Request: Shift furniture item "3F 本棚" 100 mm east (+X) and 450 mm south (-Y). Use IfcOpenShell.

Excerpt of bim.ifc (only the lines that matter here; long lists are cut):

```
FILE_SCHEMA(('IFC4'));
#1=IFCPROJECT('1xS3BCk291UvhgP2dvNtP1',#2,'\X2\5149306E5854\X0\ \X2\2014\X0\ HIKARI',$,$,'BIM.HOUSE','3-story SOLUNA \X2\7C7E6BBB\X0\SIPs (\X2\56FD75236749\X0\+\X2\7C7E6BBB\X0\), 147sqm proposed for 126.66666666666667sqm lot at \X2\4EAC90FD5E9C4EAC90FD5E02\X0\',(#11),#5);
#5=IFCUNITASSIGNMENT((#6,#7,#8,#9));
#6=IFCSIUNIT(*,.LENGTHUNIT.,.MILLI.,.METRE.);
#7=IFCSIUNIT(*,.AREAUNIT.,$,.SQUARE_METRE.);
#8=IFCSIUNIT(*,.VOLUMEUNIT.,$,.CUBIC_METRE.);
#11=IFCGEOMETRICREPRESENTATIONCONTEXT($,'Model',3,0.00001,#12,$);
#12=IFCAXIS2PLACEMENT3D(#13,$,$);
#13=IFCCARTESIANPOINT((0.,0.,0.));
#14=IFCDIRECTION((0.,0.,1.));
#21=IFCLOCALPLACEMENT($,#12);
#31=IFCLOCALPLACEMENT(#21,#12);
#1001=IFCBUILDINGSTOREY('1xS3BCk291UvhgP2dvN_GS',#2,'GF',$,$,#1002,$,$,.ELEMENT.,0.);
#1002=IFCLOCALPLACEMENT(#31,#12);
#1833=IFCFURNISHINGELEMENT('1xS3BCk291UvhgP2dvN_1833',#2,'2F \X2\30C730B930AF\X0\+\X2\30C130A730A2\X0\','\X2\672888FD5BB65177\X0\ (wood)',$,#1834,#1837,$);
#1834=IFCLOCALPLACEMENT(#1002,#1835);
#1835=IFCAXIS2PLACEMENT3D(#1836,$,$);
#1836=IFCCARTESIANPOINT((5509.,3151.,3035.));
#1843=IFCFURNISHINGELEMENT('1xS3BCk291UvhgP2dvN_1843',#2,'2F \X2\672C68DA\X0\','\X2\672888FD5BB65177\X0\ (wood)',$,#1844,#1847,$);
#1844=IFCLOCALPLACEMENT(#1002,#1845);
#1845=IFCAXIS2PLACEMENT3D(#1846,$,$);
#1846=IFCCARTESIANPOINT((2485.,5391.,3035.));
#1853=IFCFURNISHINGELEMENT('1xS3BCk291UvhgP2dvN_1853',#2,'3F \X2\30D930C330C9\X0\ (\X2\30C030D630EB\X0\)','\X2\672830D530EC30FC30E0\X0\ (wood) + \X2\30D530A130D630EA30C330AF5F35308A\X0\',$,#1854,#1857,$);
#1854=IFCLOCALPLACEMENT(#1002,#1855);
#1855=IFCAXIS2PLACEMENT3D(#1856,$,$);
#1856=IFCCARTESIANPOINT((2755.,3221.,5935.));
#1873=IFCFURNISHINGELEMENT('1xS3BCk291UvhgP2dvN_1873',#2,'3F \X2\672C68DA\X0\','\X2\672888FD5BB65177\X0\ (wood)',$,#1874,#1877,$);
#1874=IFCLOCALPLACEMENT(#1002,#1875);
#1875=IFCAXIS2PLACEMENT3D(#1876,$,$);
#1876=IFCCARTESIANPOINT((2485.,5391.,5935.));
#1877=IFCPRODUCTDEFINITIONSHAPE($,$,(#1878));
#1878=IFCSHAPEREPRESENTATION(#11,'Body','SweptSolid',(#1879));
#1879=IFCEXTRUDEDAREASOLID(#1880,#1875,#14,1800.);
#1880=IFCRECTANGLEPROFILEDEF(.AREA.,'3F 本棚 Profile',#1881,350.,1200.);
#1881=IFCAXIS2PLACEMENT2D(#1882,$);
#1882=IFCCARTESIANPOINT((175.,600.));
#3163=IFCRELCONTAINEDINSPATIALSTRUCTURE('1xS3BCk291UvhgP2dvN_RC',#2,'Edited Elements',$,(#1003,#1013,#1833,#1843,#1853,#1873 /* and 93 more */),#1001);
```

```python
import ifcopenshell
import ifcopenshell.api.geometry
import ifcopenshell.util.placement

model = ifcopenshell.open("bim.ifc")

item = model.by_guid("1xS3BCk291UvhgP2dvN_1873")
matrix = ifcopenshell.util.placement.get_local_placement(item.ObjectPlacement)
matrix[0, 3] += 100.0
matrix[1, 3] -= 450.0
ifcopenshell.api.geometry.edit_object_placement(model, product=item, matrix=matrix, is_si=False)

print(ifcopenshell.util.placement.get_local_placement(item.ObjectPlacement).round(3) + 0.0)

model.write("bim_edited.ifc")
```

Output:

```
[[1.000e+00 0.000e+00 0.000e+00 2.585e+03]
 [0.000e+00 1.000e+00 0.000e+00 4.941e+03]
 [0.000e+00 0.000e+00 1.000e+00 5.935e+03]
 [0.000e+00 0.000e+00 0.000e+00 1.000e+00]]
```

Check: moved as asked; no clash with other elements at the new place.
